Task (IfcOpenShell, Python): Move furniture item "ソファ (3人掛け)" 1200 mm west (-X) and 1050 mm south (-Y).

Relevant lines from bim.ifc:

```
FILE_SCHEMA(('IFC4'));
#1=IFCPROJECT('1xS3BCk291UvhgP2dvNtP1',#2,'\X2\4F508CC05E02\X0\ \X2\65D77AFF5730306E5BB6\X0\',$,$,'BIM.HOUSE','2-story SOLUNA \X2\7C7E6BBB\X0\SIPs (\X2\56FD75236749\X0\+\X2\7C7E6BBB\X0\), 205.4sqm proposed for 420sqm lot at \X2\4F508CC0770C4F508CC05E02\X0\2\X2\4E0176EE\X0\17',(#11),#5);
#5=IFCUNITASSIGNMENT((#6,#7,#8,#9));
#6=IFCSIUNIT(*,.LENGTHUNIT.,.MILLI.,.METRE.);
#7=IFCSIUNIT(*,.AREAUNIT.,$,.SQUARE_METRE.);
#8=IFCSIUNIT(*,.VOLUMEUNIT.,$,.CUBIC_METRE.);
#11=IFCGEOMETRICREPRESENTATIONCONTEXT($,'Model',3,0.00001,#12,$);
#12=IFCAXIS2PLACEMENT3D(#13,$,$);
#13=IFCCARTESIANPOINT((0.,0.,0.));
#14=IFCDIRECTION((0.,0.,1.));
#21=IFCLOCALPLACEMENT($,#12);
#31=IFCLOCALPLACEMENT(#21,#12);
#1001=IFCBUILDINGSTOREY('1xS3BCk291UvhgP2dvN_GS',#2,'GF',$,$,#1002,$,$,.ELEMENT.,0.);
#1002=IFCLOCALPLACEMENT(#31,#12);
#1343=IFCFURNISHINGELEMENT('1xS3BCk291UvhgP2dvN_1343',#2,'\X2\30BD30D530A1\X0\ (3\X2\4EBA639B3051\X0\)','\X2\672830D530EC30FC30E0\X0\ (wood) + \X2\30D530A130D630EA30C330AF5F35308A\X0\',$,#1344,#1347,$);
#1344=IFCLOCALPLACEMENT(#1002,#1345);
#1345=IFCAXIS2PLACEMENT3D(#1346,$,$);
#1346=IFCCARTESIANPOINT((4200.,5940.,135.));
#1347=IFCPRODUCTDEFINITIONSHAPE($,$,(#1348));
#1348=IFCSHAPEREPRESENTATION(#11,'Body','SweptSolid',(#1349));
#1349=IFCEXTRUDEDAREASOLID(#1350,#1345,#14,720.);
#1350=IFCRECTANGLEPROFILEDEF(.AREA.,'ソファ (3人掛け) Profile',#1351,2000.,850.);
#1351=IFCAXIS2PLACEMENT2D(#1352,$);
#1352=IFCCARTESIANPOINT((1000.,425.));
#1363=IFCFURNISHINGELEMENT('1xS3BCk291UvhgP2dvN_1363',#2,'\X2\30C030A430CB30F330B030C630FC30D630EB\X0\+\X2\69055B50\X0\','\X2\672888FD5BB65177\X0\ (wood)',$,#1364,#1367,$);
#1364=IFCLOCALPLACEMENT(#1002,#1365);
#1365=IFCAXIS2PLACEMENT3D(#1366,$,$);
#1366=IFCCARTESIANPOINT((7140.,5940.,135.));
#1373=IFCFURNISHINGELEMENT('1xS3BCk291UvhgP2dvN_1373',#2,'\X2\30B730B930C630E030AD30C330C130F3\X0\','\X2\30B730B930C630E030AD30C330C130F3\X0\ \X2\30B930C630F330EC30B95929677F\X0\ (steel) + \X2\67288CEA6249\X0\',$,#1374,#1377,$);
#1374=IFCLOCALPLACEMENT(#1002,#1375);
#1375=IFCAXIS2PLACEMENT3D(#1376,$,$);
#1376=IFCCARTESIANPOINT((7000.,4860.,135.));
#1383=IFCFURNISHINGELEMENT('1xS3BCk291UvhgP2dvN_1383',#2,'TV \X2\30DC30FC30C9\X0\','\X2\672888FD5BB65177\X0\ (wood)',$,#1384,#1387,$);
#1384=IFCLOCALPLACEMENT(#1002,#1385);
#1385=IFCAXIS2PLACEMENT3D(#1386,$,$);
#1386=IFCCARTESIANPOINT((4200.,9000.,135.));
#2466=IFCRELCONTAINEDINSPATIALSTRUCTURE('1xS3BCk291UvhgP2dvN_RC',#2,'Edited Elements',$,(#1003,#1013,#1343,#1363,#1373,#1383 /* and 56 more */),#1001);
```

```python
import ifcopenshell
import ifcopenshell.api.geometry
import ifcopenshell.util.placement
import ifcopenshell.util.unit

model = ifcopenshell.open("bim.ifc")
unit_scale = ifcopenshell.util.unit.calculate_unit_scale(model)

item = model.by_id(1343)
matrix = ifcopenshell.util.placement.get_local_placement(item.ObjectPlacement)
matrix[0, 3] -= 1.2 / unit_scale
matrix[1, 3] -= 1.05 / unit_scale
ifcopenshell.api.geometry.edit_object_placement(model, product=item, matrix=matrix, is_si=False)

print(ifcopenshell.util.placement.get_local_placement(item.ObjectPlacement).round(3) + 0.0)

model.write("bim_edited.ifc")
```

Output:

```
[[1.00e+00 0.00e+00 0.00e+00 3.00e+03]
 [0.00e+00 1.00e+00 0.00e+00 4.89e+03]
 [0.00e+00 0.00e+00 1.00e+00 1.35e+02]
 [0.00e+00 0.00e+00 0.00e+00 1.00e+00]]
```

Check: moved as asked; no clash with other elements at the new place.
